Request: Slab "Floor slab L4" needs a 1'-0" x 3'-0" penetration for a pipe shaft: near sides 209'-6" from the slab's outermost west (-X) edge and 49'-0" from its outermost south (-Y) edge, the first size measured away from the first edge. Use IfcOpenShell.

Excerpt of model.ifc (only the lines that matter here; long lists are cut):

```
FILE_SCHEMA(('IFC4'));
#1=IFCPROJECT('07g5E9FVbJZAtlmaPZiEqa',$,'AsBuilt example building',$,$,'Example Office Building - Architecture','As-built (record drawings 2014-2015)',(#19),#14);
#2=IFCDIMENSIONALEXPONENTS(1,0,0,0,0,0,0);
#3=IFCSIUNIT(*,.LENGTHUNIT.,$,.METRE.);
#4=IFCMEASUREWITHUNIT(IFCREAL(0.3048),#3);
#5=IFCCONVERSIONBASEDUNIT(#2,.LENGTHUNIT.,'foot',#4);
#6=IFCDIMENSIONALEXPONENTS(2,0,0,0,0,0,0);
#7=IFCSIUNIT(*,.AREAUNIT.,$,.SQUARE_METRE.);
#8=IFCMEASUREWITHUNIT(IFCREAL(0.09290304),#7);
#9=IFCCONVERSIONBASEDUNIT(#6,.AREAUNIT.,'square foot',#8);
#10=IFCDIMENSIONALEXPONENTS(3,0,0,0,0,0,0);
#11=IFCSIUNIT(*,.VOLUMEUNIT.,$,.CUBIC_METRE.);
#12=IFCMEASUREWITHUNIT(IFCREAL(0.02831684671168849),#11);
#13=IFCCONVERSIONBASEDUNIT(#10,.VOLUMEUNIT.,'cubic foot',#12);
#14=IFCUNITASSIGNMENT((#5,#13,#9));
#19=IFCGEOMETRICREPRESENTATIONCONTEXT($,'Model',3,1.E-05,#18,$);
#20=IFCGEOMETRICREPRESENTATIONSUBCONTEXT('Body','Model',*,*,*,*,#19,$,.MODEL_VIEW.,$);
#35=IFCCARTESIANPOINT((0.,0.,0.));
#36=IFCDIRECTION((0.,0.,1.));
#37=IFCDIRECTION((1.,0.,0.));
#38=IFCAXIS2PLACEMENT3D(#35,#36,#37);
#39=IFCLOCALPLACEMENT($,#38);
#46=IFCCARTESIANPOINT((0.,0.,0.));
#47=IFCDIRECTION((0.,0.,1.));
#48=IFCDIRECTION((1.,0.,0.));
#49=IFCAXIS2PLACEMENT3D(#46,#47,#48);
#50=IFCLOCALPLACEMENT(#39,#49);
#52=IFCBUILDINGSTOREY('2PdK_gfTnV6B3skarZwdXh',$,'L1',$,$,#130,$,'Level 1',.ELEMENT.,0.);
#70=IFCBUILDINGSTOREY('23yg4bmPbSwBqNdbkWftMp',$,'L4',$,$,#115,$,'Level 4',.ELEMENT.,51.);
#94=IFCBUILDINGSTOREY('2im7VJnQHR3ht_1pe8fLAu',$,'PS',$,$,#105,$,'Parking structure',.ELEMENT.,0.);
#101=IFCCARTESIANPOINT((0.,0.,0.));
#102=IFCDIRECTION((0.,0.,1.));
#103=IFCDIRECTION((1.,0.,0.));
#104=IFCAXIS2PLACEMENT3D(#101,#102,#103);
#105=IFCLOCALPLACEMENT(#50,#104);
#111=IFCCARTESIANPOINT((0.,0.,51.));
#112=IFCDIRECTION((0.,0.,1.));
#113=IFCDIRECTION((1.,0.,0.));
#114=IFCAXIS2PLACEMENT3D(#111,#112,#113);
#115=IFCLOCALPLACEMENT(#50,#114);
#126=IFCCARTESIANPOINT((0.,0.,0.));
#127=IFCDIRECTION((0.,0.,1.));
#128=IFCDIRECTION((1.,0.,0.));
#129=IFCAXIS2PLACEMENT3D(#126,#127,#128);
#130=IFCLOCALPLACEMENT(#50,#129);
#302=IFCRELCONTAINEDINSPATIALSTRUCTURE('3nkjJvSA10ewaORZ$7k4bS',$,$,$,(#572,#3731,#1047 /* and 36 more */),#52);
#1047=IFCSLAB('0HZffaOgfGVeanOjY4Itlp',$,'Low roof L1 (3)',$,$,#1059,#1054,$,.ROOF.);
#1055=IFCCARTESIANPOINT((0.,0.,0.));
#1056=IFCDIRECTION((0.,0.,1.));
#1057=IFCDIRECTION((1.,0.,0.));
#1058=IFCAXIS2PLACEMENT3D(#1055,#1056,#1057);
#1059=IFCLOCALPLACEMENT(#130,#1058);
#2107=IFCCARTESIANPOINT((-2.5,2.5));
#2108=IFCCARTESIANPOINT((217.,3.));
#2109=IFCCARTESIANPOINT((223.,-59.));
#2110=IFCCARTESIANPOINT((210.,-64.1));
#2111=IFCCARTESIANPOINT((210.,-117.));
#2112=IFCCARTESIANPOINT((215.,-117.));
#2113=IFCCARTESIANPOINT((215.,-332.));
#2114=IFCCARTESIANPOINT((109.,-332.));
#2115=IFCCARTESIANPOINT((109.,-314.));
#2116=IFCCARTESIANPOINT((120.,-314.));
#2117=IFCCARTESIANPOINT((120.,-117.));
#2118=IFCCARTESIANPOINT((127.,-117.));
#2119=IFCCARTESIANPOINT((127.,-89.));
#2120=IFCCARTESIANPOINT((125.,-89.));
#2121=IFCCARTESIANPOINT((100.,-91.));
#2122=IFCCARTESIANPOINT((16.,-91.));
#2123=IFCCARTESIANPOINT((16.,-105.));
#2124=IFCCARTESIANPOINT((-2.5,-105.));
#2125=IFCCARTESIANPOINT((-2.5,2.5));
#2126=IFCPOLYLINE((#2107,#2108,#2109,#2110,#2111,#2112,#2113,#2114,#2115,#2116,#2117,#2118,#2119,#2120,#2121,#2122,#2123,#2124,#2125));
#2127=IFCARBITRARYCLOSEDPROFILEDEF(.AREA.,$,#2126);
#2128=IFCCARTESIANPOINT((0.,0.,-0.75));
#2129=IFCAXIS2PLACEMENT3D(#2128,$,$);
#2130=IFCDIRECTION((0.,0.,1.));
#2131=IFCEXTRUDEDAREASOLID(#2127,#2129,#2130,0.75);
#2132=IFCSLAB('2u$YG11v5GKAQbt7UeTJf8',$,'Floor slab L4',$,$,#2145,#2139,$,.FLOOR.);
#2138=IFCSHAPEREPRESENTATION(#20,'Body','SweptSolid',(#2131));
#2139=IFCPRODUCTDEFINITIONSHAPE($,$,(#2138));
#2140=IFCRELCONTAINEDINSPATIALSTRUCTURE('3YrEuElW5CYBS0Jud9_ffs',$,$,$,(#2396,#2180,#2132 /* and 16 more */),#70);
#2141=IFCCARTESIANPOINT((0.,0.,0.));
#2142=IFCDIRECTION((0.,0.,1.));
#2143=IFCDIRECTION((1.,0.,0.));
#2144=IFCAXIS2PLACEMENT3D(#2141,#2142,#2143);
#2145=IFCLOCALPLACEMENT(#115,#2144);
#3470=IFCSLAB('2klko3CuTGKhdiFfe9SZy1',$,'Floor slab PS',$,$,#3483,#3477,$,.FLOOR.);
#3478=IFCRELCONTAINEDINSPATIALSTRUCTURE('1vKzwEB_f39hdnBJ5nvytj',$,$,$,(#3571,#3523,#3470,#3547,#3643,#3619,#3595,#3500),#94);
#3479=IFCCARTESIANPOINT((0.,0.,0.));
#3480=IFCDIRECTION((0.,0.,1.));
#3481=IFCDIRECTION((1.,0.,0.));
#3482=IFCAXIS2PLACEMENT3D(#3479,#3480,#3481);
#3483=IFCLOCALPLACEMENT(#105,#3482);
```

```python
import numpy as np
import ifcopenshell
import ifcopenshell.api.feature
import ifcopenshell.api.geometry
import ifcopenshell.api.root
import ifcopenshell.geom
import ifcopenshell.util.placement
import ifcopenshell.util.representation
import ifcopenshell.util.shape
import ifcopenshell.util.unit

model = ifcopenshell.open("model.ifc")
unit_scale = ifcopenshell.util.unit.calculate_unit_scale(model)
settings = ifcopenshell.geom.settings()


def volume(element):
    """Net volume in cubic metres, openings subtracted."""
    shape = ifcopenshell.geom.create_shape(settings, element)
    return ifcopenshell.util.shape.get_volume(shape.geometry)


slab = model.by_id(2132)
before = volume(slab)

# Extent in the slab's own axes, in metres. The edges named are its -X and -Y sides.
slab_shape = ifcopenshell.geom.create_shape(settings, slab)
vertices = ifcopenshell.util.shape.get_vertices(slab_shape.geometry)
x_min, y_min, bottom = vertices.min(axis=0)
top = vertices[:, 2].max()

opening = ifcopenshell.api.root.create_entity(model, ifc_class="IfcOpeningElement", name="Pipe shaft opening", predefined_type="OPENING")
context = ifcopenshell.util.representation.get_context(model, "Model", "Body", "MODEL_VIEW")
width, depth = 0.3048, 0.9144
outline = [(0.0, 0.0), (width, 0.0), (width, depth), (0.0, depth), (0.0, 0.0)]
# Overshoot both faces by 50 mm so the cut is clean.
shape = ifcopenshell.api.geometry.add_slab_representation(
    model, context=context, depth=top - bottom + 0.1, polyline=outline
)
ifcopenshell.api.geometry.assign_representation(model, product=opening, representation=shape)

matrix = ifcopenshell.util.placement.get_local_placement(slab.ObjectPlacement)
matrix[:, 3] = matrix @ np.append(np.array([x_min + 63.8556, y_min + 14.9352, bottom - 0.05]) / unit_scale, 1.0)
ifcopenshell.api.geometry.edit_object_placement(model, product=opening, matrix=matrix, is_si=False)
ifcopenshell.api.feature.add_feature(model, feature=opening, element=slab)

after = volume(slab)

print(f"slab volume {before:.3f} -> {after:.3f} m3")

model.write("model_edited.ifc")
```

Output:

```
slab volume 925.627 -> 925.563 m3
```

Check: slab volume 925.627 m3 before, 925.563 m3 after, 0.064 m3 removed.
